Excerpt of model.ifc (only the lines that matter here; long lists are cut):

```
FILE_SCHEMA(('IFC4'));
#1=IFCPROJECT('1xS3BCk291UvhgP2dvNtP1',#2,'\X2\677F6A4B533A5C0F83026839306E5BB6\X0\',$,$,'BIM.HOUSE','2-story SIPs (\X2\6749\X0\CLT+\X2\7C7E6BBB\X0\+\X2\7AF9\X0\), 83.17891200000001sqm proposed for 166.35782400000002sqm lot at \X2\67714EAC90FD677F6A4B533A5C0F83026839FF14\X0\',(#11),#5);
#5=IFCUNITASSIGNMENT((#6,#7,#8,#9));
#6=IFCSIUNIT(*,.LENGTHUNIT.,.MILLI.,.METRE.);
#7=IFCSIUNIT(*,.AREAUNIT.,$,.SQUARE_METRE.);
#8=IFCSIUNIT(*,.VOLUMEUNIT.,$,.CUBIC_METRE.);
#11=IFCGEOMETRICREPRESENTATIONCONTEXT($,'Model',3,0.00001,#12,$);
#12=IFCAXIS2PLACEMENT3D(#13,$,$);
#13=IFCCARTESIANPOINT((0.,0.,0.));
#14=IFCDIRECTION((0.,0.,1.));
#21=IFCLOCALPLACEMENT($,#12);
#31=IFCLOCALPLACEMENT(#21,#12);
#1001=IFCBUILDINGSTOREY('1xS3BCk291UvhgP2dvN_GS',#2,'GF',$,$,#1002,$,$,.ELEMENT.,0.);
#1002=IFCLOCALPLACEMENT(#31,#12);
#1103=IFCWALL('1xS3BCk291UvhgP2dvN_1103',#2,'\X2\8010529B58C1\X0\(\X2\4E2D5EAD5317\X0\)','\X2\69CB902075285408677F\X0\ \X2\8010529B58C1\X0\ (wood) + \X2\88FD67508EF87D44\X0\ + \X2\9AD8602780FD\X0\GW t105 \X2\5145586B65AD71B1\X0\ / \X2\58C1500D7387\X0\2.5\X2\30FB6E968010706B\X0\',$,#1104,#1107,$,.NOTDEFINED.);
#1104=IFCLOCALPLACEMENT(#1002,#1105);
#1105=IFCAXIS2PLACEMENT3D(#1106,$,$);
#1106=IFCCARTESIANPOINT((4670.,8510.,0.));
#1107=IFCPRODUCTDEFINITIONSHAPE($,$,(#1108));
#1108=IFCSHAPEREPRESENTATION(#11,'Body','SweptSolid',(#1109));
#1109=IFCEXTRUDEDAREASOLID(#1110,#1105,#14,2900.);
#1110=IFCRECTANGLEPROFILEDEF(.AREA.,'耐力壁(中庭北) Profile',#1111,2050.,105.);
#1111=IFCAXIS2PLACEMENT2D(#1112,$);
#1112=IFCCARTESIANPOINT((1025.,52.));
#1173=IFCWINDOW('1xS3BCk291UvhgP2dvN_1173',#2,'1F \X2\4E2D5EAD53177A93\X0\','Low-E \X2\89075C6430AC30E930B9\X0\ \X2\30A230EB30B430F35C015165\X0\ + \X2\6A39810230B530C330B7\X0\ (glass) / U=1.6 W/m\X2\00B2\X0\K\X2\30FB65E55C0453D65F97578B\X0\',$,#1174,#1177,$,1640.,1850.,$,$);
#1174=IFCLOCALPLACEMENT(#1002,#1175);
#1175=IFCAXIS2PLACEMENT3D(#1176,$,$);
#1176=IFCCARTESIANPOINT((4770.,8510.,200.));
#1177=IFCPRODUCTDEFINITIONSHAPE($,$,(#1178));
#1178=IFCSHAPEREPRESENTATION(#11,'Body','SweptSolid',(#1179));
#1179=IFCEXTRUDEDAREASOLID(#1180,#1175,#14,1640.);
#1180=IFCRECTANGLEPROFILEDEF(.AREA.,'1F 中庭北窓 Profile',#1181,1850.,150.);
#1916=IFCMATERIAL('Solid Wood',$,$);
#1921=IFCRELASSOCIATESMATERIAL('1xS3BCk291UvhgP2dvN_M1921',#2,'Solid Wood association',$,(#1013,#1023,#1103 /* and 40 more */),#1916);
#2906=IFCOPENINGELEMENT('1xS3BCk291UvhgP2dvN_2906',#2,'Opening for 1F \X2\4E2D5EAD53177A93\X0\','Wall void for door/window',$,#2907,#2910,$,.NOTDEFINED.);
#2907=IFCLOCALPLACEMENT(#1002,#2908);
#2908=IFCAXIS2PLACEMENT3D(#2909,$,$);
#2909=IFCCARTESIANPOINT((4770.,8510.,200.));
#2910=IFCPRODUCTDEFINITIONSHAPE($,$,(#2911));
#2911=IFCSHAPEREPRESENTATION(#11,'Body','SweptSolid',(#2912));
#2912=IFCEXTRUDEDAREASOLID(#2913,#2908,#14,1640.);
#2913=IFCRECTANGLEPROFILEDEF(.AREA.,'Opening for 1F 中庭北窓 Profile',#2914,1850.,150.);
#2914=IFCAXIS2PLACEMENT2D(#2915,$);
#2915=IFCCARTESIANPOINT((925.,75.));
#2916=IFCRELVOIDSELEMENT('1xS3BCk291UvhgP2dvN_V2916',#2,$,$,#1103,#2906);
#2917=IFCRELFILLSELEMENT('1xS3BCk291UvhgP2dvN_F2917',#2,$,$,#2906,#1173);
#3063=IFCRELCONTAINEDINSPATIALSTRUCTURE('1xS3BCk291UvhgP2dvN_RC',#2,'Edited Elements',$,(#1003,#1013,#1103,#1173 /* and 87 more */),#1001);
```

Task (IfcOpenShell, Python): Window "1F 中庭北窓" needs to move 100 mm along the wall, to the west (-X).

```python
import ifcopenshell
import ifcopenshell.api.geometry
import ifcopenshell.util.placement
import ifcopenshell.util.unit

model = ifcopenshell.open("model.ifc")
unit_scale = ifcopenshell.util.unit.calculate_unit_scale(model)

window = model.by_guid("1xS3BCk291UvhgP2dvN_1173")
opening = window.FillsVoids[0].RelatingOpeningElement
wall = opening.VoidsElements[0].RelatingBuildingElement

wall_matrix = ifcopenshell.util.placement.get_local_placement(wall.ObjectPlacement)
shift = wall_matrix[:3, 0] * -0.1 / unit_scale
before = ifcopenshell.util.placement.get_local_placement(window.ObjectPlacement)[:3, 3].copy()

# The window is not placed relative to its opening, so move both.
for product in (opening, window):
    matrix = ifcopenshell.util.placement.get_local_placement(product.ObjectPlacement)
    matrix[:3, 3] += shift
    ifcopenshell.api.geometry.edit_object_placement(model, product=product, matrix=matrix, is_si=False)

after = ifcopenshell.util.placement.get_local_placement(window.ObjectPlacement)[:3, 3]
print("window moved by", (after - before).round(3) + 0.0)

model.write("model_v2.ifc")
```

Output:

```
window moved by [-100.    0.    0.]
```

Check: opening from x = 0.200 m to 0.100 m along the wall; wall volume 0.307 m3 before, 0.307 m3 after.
